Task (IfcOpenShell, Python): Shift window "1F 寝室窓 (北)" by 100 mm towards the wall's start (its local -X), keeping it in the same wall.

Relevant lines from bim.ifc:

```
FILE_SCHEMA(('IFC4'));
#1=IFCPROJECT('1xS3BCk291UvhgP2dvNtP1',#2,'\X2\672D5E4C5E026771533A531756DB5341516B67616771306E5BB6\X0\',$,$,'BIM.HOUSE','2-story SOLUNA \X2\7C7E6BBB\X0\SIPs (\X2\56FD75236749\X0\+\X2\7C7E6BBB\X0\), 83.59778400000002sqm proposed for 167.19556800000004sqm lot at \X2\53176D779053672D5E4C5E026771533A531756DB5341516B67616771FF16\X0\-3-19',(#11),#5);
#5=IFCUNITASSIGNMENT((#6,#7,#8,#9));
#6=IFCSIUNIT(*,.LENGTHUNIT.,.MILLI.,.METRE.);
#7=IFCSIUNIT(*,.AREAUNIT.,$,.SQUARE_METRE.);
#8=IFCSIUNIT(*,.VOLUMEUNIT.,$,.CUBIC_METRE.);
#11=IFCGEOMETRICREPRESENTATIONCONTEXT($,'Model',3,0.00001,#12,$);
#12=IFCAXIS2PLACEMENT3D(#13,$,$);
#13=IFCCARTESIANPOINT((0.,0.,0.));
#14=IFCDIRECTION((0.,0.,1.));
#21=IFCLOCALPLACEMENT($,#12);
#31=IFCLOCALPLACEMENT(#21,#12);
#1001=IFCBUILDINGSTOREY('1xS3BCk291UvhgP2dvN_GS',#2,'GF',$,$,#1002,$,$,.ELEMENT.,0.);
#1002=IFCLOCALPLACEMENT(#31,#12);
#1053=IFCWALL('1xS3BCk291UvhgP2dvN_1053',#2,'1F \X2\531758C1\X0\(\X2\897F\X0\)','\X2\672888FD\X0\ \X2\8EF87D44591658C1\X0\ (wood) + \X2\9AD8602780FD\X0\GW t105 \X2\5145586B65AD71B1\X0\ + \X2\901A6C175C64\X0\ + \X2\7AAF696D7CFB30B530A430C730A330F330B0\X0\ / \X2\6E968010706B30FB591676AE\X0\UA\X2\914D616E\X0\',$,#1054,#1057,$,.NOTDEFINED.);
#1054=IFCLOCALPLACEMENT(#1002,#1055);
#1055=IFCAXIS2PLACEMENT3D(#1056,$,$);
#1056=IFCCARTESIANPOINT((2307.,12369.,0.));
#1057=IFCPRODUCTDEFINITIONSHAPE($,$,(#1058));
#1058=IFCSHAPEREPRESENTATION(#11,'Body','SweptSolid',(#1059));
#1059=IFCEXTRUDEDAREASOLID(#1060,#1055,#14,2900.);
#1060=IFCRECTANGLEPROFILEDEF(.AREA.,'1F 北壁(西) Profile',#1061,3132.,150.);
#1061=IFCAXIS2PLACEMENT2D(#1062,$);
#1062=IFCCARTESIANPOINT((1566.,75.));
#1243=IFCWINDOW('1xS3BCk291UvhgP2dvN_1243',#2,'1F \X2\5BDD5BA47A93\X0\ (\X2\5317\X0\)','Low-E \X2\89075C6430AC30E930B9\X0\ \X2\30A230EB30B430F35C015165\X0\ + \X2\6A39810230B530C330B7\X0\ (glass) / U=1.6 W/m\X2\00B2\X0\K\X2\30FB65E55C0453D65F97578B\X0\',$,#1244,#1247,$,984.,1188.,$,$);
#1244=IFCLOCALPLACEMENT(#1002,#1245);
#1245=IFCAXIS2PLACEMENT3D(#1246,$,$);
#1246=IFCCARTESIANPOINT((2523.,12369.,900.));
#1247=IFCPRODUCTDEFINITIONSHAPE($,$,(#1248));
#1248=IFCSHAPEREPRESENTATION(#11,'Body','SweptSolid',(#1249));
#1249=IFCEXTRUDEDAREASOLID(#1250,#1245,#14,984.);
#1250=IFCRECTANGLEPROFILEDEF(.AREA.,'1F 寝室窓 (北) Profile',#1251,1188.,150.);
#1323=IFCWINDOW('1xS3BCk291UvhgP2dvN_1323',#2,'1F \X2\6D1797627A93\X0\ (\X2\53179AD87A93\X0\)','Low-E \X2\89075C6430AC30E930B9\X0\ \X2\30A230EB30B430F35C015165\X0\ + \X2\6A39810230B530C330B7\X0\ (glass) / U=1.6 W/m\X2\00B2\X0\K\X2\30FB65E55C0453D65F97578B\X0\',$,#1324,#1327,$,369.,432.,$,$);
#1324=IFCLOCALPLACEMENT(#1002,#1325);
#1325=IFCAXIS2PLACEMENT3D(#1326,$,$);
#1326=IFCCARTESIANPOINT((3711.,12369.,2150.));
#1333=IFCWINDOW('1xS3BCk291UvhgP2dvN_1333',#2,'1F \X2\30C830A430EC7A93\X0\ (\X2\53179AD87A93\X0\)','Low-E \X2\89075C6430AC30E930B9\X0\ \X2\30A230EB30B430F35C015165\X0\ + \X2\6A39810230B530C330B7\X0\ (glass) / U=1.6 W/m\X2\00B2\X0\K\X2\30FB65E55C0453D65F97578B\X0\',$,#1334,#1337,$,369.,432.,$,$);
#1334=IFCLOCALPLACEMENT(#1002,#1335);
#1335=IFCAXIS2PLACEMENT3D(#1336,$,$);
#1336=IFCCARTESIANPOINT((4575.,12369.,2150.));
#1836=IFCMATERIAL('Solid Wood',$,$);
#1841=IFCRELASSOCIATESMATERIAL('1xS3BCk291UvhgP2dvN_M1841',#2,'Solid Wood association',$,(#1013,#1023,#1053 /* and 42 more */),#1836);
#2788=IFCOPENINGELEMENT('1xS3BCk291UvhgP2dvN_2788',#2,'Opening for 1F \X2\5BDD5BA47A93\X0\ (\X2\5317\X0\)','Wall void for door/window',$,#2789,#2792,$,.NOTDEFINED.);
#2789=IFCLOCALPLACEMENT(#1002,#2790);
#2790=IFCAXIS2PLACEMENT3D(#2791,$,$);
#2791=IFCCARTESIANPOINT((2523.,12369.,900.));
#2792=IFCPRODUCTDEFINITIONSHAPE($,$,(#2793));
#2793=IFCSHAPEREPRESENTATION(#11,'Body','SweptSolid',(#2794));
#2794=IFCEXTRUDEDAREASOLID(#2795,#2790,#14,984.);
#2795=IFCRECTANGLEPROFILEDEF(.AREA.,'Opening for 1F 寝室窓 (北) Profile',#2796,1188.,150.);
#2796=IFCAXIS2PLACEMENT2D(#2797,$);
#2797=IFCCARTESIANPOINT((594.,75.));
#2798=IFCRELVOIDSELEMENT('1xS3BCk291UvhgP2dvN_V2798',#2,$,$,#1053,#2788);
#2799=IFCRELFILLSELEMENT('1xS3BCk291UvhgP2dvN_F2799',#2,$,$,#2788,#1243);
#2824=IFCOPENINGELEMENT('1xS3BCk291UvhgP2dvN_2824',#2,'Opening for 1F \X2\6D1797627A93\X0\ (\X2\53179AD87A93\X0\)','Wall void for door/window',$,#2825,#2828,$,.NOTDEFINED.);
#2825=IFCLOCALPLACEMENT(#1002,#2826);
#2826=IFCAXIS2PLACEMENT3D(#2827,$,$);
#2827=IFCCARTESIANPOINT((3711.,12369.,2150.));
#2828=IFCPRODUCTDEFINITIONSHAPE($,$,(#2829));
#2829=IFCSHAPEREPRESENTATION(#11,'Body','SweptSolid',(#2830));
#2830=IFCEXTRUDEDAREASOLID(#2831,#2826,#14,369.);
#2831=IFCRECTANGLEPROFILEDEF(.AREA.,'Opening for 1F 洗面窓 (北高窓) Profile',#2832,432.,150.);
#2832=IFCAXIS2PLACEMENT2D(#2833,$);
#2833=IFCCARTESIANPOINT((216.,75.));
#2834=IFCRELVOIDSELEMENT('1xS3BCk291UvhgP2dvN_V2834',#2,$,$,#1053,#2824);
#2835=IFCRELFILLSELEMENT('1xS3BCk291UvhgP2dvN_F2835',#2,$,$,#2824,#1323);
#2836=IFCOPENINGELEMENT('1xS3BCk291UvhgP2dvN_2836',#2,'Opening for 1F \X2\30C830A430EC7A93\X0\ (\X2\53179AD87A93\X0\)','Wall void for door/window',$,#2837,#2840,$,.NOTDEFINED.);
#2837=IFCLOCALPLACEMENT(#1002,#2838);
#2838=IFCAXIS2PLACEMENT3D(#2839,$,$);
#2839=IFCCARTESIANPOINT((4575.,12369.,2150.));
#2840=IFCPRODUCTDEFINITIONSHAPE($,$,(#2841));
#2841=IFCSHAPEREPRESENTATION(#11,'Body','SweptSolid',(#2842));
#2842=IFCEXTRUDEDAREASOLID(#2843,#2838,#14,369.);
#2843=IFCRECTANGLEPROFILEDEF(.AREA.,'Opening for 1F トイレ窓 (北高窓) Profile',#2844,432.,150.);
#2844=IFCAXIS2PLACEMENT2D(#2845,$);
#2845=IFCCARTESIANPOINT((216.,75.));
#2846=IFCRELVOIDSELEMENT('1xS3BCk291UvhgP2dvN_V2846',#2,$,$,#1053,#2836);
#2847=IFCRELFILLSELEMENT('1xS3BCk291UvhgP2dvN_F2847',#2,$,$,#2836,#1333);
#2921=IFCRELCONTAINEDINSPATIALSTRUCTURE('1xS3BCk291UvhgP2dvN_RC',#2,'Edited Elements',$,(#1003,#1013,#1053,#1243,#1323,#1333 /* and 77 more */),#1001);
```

```python
import ifcopenshell
import ifcopenshell.api.geometry
import ifcopenshell.util.placement
import ifcopenshell.util.unit

model = ifcopenshell.open("bim.ifc")
unit_scale = ifcopenshell.util.unit.calculate_unit_scale(model)

window = model.by_guid("1xS3BCk291UvhgP2dvN_1243")
opening = window.FillsVoids[0].RelatingOpeningElement
wall = opening.VoidsElements[0].RelatingBuildingElement

wall_matrix = ifcopenshell.util.placement.get_local_placement(wall.ObjectPlacement)
shift = wall_matrix[:3, 0] * -0.1 / unit_scale
before = ifcopenshell.util.placement.get_local_placement(window.ObjectPlacement)[:3, 3].copy()

# The window is not placed relative to its opening, so move both.
for product in (opening, window):
    matrix = ifcopenshell.util.placement.get_local_placement(product.ObjectPlacement)
    matrix[:3, 3] += shift
    ifcopenshell.api.geometry.edit_object_placement(model, product=product, matrix=matrix, is_si=False)

after = ifcopenshell.util.placement.get_local_placement(window.ObjectPlacement)[:3, 3]
print("window moved by", (after - before).round(3) + 0.0)

model.write("bim_updated.ifc")
```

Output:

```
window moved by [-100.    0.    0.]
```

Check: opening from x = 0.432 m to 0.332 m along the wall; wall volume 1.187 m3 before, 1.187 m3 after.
